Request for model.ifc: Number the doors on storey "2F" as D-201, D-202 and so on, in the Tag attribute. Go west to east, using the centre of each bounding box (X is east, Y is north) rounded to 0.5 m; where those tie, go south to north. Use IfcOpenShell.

First a look at what the model holds.

```python
import ifcopenshell
import ifcopenshell.util.element
import ifcopenshell.util.placement

model = ifcopenshell.open("model.ifc")
print(model.schema)
storey = next(s for s in model.by_type("IfcBuildingStorey") if s.Name == "2F")
doors = [e for e in ifcopenshell.util.element.get_decomposition(storey) if e.is_a("IfcDoor")]
for e in sorted(doors, key=lambda e: e.id()):
    origin = ifcopenshell.util.placement.get_local_placement(e.ObjectPlacement)[:3, 3]
    print(e.id(), e.Tag, e.Name, origin.round(2) + 0.0, sep=" | ")
```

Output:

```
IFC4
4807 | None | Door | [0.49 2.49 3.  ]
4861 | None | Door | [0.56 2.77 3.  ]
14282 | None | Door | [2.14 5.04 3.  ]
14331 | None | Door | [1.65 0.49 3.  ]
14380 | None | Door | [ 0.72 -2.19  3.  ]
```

```python
import ifcopenshell
import ifcopenshell.geom
import ifcopenshell.util.element
import ifcopenshell.util.shape

model = ifcopenshell.open("model.ifc")
settings = ifcopenshell.geom.settings()
settings.set("use-world-coords", True)


def centre(element):
    shape = ifcopenshell.geom.create_shape(settings, element)
    return ifcopenshell.util.shape.get_bbox_centroid(shape.geometry)


storey = next(s for s in model.by_type("IfcBuildingStorey") if s.Name == "2F")
doors = [e for e in ifcopenshell.util.element.get_decomposition(storey) if e.is_a("IfcDoor")]

# Insertion points can sit at a corner or the storey origin, so sort by the geometry (in metres).
centres = {e: centre(e) for e in doors}
doors.sort(key=lambda e: (round(centres[e][0] / 0.5), centres[e][1]))

for i, e in enumerate(doors, start=1):
    number = f"D-2{i:02d}"
    e.Tag = number
    print(e.id(), number)

model.write("model_rev.ifc")
```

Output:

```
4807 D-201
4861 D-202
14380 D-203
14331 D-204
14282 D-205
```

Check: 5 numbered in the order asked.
